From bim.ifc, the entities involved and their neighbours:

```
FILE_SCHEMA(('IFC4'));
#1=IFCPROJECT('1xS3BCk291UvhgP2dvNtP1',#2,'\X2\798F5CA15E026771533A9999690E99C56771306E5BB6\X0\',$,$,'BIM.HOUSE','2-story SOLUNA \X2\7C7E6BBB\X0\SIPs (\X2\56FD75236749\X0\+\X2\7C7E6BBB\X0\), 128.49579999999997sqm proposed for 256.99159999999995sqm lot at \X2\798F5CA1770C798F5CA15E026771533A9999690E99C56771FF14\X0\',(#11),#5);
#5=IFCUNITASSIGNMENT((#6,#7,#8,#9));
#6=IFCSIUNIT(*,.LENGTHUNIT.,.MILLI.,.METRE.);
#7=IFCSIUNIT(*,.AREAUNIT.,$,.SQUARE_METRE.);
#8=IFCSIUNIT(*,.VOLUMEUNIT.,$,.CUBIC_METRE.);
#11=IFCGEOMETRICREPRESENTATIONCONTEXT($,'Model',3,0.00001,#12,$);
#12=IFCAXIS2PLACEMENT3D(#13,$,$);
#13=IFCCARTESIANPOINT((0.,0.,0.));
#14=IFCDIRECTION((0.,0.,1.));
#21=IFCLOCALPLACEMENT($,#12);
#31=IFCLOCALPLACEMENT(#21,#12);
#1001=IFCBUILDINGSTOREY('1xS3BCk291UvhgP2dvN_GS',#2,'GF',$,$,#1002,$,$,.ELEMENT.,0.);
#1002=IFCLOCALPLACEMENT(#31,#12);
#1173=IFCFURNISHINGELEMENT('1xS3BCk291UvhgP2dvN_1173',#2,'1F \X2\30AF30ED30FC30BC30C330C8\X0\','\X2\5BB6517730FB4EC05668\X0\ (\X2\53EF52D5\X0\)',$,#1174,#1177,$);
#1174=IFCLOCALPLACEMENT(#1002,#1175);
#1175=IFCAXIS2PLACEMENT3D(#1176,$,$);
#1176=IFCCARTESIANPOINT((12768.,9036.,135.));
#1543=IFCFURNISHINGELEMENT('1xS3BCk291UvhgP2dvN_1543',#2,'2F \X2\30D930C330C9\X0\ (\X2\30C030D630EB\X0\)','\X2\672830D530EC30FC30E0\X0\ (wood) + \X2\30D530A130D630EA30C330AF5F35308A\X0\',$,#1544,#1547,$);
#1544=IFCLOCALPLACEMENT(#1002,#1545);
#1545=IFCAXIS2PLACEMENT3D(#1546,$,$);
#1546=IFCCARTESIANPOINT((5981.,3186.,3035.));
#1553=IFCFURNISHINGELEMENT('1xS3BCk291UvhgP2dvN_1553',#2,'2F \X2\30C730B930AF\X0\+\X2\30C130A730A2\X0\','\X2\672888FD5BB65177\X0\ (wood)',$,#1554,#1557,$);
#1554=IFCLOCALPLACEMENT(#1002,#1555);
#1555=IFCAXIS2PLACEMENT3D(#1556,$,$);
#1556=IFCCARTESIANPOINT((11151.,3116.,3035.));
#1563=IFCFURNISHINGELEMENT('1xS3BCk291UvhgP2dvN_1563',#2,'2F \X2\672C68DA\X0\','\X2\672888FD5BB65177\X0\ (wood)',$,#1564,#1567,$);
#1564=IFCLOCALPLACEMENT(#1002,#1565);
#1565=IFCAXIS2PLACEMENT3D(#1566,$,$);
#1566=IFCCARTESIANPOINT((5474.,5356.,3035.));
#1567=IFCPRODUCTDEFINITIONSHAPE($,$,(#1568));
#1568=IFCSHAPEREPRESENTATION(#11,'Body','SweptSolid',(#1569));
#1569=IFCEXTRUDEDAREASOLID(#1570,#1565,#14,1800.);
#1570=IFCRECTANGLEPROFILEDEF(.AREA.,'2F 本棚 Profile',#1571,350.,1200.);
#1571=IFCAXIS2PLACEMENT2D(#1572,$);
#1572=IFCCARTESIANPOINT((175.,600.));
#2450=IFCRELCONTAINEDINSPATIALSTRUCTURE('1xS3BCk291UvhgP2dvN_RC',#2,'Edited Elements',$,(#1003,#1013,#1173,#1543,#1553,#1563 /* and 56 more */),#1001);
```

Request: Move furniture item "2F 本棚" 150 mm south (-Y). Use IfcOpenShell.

```python
import ifcopenshell
import ifcopenshell.api.geometry
import ifcopenshell.util.placement
import ifcopenshell.util.unit

model = ifcopenshell.open("bim.ifc")
unit_scale = ifcopenshell.util.unit.calculate_unit_scale(model)

item = model.by_id(1563)
matrix = ifcopenshell.util.placement.get_local_placement(item.ObjectPlacement)
matrix[1, 3] -= 0.15 / unit_scale
ifcopenshell.api.geometry.edit_object_placement(model, product=item, matrix=matrix, is_si=False)

print(ifcopenshell.util.placement.get_local_placement(item.ObjectPlacement).round(3) + 0.0)

model.write("bim-out.ifc")
```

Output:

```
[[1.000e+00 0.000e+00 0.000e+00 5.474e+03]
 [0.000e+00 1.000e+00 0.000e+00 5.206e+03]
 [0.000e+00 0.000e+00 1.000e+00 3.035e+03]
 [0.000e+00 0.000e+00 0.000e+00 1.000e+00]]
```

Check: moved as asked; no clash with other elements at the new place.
